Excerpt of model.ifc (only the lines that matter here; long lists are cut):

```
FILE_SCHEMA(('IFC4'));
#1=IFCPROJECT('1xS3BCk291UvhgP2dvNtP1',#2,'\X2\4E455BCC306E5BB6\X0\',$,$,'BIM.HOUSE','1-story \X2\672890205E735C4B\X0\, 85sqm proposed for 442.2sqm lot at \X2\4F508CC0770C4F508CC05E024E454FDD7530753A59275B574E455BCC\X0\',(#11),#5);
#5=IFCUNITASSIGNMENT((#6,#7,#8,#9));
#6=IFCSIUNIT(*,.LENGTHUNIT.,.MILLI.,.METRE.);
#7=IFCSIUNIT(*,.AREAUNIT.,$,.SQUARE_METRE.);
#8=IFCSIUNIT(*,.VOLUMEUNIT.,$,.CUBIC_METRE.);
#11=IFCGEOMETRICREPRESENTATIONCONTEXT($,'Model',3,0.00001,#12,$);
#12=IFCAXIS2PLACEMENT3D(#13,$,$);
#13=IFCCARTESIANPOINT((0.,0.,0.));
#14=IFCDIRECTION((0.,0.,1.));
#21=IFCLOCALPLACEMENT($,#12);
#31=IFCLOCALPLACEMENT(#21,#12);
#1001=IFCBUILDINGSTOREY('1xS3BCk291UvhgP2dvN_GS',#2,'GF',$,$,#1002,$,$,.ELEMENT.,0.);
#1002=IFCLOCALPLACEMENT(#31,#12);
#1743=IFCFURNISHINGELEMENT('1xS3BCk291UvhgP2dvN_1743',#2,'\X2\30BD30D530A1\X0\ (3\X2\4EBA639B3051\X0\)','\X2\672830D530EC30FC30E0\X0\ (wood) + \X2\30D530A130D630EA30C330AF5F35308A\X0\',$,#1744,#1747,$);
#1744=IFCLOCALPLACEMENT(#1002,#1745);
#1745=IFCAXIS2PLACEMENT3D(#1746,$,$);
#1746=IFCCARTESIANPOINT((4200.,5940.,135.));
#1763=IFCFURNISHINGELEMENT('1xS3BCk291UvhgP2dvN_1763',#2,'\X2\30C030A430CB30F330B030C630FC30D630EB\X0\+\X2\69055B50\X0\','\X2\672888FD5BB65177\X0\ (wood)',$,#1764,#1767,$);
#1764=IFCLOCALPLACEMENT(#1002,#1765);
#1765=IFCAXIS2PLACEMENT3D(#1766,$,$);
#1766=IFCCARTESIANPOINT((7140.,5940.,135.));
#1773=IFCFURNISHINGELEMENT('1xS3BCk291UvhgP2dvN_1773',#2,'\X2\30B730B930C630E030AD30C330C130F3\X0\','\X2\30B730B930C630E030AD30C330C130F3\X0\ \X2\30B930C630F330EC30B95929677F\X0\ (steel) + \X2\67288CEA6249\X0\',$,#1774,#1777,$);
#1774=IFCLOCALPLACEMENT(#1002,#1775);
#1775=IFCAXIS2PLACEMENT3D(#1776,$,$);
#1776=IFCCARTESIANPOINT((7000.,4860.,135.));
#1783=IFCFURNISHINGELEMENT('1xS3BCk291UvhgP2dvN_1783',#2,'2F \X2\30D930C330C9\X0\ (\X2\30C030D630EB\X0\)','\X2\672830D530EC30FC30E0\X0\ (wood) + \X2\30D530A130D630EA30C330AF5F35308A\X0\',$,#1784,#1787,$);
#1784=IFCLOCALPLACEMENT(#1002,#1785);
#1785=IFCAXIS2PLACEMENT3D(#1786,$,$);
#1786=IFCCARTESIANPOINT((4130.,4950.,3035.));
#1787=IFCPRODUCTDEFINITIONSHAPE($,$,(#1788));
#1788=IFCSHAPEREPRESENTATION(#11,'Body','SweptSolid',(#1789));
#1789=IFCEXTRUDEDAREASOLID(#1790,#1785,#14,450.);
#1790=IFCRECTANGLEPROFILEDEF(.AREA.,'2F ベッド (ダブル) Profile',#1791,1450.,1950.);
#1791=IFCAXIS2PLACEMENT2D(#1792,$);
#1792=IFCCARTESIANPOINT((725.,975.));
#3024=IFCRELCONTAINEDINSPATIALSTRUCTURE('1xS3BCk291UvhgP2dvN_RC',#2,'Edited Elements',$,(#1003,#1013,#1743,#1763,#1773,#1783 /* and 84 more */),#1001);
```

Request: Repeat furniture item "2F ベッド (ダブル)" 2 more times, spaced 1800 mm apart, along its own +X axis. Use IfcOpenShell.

```python
import ifcopenshell
import ifcopenshell.api.geometry
import ifcopenshell.api.root
import ifcopenshell.util.element
import ifcopenshell.util.placement
import ifcopenshell.util.unit

model = ifcopenshell.open("model.ifc")
unit_scale = ifcopenshell.util.unit.calculate_unit_scale(model)


def reuse_history(source, copy):
    """copy_class also copies each property set's owner history, people and application; keep the originals."""
    for rel in copy.IsDefinedBy:
        if rel.is_a("IfcRelDefinesByProperties") and (history := rel.RelatingPropertyDefinition.OwnerHistory):
            rel.RelatingPropertyDefinition.OwnerHistory = source.OwnerHistory
            ifcopenshell.util.element.remove_deep2(model, history)


source = model.by_id(1783)
base = ifcopenshell.util.placement.get_local_placement(source.ObjectPlacement)
step = base[:3, 0] * 1.8 / unit_scale

for i in range(1, 3):
    copy = ifcopenshell.api.root.copy_class(model, product=source)
    copy.Representation = ifcopenshell.util.element.copy_deep(
        model, source.Representation, exclude=["IfcGeometricRepresentationContext", "IfcRepresentationMap"]
    )
    reuse_history(source, copy)
    matrix = base.copy()
    matrix[:3, 3] += i * step
    print("added at", matrix[:3, 3].round(3) + 0.0)
    ifcopenshell.api.geometry.edit_object_placement(model, product=copy, matrix=matrix, is_si=False)

model.write("model-out.ifc")
```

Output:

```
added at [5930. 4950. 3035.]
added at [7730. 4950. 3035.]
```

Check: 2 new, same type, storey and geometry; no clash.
